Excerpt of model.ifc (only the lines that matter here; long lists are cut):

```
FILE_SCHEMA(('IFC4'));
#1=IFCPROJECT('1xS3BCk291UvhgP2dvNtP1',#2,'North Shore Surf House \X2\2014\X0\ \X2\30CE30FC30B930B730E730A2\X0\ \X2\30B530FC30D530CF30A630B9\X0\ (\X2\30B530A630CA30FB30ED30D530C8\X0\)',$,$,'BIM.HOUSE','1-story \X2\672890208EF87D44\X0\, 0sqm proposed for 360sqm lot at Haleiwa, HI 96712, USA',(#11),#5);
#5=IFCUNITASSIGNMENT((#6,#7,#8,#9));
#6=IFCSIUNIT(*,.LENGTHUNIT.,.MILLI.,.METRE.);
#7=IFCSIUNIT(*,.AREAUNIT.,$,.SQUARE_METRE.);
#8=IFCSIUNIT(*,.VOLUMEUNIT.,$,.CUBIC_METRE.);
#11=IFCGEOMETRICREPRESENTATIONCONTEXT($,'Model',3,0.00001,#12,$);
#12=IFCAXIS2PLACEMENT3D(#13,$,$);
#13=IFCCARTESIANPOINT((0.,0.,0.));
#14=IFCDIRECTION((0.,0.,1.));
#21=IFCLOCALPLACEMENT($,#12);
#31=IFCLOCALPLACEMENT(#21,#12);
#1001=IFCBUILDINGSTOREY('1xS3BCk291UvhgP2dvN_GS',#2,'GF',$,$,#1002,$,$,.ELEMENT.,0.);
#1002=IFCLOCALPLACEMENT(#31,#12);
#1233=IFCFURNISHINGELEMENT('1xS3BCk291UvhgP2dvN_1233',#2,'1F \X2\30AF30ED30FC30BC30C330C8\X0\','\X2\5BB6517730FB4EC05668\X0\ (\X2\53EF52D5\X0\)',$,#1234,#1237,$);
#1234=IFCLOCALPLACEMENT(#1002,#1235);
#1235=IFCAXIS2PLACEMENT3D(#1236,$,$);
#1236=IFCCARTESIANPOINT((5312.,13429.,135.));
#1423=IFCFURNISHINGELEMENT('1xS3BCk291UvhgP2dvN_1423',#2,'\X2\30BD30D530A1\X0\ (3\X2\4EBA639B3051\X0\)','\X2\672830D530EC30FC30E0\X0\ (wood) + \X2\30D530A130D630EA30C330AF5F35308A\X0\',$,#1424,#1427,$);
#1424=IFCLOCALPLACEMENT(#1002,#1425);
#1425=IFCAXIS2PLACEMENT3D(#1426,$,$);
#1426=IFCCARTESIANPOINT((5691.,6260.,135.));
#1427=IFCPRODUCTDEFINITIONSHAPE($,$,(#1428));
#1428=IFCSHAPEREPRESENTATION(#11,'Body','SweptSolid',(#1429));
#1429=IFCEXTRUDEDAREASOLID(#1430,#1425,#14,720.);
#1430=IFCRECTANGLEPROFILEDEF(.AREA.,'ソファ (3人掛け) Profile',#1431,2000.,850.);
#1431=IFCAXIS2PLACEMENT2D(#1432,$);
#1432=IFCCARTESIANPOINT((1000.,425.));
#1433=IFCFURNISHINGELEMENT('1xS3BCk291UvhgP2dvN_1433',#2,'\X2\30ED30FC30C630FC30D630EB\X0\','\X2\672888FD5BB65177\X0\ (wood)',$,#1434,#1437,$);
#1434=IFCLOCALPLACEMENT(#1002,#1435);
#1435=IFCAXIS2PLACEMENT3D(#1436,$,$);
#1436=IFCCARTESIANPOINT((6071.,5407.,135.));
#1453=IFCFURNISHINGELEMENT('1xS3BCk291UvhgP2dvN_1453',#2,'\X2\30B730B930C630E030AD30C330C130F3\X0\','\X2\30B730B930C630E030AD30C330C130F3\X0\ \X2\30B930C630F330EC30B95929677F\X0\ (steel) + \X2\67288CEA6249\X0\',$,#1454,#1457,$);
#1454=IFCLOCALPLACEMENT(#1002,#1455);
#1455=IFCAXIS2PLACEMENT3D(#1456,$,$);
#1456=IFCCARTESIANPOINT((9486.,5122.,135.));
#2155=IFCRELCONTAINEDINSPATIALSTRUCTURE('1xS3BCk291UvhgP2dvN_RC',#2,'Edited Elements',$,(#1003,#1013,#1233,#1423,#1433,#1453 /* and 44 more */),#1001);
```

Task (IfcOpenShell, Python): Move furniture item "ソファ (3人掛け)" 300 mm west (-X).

```python
import ifcopenshell
import ifcopenshell.api.geometry
import ifcopenshell.util.placement
import ifcopenshell.util.unit

model = ifcopenshell.open("model.ifc")
unit_scale = ifcopenshell.util.unit.calculate_unit_scale(model)

item = model.by_id(1423)
matrix = ifcopenshell.util.placement.get_local_placement(item.ObjectPlacement)
matrix[0, 3] -= 0.3 / unit_scale
ifcopenshell.api.geometry.edit_object_placement(model, product=item, matrix=matrix, is_si=False)

print(ifcopenshell.util.placement.get_local_placement(item.ObjectPlacement).round(3) + 0.0)

model.write("model_updated.ifc")
```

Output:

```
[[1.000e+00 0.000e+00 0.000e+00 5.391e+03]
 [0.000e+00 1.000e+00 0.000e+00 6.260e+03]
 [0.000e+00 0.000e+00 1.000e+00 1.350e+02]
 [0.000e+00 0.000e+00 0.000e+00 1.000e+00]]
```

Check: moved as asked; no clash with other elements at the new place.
